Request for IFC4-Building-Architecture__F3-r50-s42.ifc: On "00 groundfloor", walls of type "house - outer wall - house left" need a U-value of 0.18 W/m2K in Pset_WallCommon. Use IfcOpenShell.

First a look at what the model holds.

```python
import ifcopenshell
import ifcopenshell.util.element

model = ifcopenshell.open("IFC4-Building-Architecture__F3-r50-s42.ifc")
print(model.schema)
storey = next(s for s in model.by_type("IfcBuildingStorey") if s.Name == "00 groundfloor")
walls = [e for e in ifcopenshell.util.element.get_decomposition(storey) if e.is_a("IfcWall")]
seen = {}
for e in walls:
    element_type = ifcopenshell.util.element.get_type(e)
    key = (element_type.Name if element_type != e and element_type else None, ifcopenshell.util.element.get_pset(e, "Pset_WallCommon", "ThermalTransmittance"))
    seen[key] = seen.get(key, 0) + 1
for (name, value), count in sorted(seen.items(), key=str):
    print(count, "x", name, "|", value)
```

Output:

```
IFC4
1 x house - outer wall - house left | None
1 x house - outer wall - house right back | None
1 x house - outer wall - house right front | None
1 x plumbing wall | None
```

```python
import ifcopenshell
import ifcopenshell.api.pset
import ifcopenshell.util.element

model = ifcopenshell.open("IFC4-Building-Architecture__F3-r50-s42.ifc")

storey = next(s for s in model.by_type("IfcBuildingStorey") if s.Name == "00 groundfloor")
walls = [e for e in ifcopenshell.util.element.get_decomposition(storey) if e.is_a("IfcWall")]

count = 0
for e in walls:
    element_type = ifcopenshell.util.element.get_type(e)
    if element_type in (None, e) or element_type.Name != "house - outer wall - house left":
        continue
    # add_pset returns the element's existing set when there is one.
    pset = ifcopenshell.api.pset.add_pset(model, product=e, name="Pset_WallCommon")
    ifcopenshell.api.pset.edit_pset(model, pset=pset, properties={"ThermalTransmittance": 0.18})
    count += 1

print(count, "walls updated")

model.write("IFC4-Building-Architecture__F3-r50-s42_v2.ifc")
```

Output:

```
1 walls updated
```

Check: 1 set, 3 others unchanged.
